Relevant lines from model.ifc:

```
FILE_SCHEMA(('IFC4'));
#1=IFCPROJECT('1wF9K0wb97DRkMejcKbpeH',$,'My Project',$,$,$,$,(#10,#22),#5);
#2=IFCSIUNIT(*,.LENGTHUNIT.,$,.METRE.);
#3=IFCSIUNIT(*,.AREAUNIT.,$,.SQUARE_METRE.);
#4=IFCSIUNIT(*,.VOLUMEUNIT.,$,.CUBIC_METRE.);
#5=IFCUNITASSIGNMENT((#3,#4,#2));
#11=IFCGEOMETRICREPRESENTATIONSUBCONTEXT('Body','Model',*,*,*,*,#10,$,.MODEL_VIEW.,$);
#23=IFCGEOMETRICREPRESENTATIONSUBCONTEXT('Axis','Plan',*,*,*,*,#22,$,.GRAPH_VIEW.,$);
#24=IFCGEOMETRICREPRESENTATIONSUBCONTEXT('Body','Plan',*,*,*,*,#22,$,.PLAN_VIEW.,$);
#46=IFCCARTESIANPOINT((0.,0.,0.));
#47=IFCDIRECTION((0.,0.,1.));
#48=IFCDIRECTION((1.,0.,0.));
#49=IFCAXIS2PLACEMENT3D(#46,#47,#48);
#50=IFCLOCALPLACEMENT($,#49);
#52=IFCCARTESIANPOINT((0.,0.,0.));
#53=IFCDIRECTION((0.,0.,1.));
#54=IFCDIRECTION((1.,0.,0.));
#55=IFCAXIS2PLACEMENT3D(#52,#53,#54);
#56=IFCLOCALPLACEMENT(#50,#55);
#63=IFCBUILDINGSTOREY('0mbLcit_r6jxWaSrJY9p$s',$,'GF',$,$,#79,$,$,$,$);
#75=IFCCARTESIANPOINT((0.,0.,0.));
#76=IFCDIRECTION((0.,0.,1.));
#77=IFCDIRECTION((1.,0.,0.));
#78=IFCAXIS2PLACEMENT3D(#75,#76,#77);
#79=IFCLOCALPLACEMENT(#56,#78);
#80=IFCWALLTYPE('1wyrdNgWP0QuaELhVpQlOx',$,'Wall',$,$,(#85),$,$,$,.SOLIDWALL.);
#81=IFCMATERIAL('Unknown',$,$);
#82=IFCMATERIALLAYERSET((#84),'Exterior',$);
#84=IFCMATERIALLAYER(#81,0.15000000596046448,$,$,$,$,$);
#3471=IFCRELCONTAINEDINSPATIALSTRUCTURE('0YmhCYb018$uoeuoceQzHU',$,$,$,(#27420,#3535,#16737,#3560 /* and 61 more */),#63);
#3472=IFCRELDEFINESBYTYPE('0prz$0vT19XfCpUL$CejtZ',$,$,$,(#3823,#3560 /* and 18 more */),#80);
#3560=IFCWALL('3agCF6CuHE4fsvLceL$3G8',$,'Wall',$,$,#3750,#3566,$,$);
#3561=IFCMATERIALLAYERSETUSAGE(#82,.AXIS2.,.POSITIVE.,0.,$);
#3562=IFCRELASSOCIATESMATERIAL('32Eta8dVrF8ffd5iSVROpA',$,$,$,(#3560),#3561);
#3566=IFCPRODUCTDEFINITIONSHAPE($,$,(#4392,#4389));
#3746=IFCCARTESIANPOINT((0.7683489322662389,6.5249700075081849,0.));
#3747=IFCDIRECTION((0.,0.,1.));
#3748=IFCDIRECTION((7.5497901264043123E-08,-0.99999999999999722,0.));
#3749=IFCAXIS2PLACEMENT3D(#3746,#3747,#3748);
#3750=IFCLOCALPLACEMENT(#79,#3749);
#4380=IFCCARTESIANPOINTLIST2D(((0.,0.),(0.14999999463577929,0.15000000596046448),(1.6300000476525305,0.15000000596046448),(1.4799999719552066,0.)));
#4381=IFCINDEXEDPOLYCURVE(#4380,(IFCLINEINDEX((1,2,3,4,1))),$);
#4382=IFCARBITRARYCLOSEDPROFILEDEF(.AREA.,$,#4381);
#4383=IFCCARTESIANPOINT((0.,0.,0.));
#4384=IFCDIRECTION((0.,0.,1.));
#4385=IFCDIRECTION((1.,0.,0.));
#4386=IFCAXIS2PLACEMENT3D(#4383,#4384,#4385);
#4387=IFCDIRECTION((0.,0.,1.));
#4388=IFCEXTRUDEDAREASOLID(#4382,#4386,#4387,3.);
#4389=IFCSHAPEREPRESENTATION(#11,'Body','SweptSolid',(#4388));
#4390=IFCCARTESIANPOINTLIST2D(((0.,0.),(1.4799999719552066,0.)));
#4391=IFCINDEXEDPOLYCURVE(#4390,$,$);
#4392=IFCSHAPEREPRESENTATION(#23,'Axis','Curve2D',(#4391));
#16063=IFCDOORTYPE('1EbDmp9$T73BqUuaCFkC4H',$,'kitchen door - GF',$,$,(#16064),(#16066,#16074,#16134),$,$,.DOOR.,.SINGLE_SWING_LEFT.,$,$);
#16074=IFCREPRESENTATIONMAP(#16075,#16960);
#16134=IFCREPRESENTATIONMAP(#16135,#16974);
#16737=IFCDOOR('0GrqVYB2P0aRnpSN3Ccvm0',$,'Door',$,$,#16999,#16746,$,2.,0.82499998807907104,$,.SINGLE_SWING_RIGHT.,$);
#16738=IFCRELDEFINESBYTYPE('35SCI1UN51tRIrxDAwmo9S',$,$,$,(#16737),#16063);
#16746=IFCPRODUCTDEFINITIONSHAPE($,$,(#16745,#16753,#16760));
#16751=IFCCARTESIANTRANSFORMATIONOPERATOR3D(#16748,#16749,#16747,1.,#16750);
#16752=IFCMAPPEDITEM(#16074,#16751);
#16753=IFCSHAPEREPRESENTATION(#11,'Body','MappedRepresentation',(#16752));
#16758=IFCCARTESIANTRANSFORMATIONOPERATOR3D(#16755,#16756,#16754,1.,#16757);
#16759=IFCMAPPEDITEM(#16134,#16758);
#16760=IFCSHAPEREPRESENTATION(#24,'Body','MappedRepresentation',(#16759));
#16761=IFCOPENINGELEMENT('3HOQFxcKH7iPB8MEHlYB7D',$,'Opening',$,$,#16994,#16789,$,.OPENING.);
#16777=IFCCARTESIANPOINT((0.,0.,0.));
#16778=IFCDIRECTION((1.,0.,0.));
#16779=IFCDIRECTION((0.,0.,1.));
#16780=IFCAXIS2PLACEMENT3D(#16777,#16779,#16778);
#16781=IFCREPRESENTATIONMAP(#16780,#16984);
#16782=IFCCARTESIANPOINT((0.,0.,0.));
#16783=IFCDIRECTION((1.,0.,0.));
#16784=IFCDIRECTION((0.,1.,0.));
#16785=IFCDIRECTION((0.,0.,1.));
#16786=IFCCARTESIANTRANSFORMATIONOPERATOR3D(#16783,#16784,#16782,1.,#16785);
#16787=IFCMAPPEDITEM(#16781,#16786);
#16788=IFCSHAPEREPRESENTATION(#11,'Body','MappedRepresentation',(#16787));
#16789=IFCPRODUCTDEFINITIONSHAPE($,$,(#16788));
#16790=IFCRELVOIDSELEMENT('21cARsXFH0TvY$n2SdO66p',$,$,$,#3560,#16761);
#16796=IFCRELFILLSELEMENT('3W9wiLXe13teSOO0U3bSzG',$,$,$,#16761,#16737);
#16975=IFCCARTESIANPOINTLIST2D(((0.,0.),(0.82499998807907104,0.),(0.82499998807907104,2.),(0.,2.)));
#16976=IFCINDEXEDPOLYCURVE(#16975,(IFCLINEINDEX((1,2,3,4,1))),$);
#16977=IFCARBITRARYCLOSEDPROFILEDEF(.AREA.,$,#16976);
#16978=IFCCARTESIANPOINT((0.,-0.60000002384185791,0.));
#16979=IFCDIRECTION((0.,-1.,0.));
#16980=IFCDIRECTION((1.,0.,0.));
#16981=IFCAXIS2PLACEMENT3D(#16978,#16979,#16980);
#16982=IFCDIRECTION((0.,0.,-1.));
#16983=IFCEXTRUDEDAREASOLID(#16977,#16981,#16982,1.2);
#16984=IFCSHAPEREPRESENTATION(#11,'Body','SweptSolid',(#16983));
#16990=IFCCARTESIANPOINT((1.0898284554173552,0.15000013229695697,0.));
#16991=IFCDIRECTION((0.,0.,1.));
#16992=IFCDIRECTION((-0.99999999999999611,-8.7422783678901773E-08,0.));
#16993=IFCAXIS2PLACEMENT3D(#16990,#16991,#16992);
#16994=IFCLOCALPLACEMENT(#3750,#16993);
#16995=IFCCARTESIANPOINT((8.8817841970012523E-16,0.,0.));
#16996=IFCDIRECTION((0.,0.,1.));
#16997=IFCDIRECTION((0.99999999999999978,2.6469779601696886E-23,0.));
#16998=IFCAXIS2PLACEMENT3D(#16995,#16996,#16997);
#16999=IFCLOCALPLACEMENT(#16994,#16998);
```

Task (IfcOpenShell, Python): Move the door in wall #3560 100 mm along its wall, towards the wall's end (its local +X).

```python
import ifcopenshell
import ifcopenshell.api.geometry
import ifcopenshell.util.placement

model = ifcopenshell.open("model.ifc")

door = model.by_guid("0GrqVYB2P0aRnpSN3Ccvm0")
opening = door.FillsVoids[0].RelatingOpeningElement
wall = opening.VoidsElements[0].RelatingBuildingElement

wall_matrix = ifcopenshell.util.placement.get_local_placement(wall.ObjectPlacement)
shift = wall_matrix[:3, 0] * 0.1
before = ifcopenshell.util.placement.get_local_placement(door.ObjectPlacement)[:3, 3].copy()

# The door is placed relative to its opening, so it follows when the opening moves.
matrix = ifcopenshell.util.placement.get_local_placement(opening.ObjectPlacement)
matrix[:3, 3] += shift
ifcopenshell.api.geometry.edit_object_placement(
    model, product=opening, matrix=matrix, is_si=False, should_transform_children=True
)

after = ifcopenshell.util.placement.get_local_placement(door.ObjectPlacement)[:3, 3]
print("door moved by", (after - before).round(3) + 0.0)

model.write("model-out.ifc")
```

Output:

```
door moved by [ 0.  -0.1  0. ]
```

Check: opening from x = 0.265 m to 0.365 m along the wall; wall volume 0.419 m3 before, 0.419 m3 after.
